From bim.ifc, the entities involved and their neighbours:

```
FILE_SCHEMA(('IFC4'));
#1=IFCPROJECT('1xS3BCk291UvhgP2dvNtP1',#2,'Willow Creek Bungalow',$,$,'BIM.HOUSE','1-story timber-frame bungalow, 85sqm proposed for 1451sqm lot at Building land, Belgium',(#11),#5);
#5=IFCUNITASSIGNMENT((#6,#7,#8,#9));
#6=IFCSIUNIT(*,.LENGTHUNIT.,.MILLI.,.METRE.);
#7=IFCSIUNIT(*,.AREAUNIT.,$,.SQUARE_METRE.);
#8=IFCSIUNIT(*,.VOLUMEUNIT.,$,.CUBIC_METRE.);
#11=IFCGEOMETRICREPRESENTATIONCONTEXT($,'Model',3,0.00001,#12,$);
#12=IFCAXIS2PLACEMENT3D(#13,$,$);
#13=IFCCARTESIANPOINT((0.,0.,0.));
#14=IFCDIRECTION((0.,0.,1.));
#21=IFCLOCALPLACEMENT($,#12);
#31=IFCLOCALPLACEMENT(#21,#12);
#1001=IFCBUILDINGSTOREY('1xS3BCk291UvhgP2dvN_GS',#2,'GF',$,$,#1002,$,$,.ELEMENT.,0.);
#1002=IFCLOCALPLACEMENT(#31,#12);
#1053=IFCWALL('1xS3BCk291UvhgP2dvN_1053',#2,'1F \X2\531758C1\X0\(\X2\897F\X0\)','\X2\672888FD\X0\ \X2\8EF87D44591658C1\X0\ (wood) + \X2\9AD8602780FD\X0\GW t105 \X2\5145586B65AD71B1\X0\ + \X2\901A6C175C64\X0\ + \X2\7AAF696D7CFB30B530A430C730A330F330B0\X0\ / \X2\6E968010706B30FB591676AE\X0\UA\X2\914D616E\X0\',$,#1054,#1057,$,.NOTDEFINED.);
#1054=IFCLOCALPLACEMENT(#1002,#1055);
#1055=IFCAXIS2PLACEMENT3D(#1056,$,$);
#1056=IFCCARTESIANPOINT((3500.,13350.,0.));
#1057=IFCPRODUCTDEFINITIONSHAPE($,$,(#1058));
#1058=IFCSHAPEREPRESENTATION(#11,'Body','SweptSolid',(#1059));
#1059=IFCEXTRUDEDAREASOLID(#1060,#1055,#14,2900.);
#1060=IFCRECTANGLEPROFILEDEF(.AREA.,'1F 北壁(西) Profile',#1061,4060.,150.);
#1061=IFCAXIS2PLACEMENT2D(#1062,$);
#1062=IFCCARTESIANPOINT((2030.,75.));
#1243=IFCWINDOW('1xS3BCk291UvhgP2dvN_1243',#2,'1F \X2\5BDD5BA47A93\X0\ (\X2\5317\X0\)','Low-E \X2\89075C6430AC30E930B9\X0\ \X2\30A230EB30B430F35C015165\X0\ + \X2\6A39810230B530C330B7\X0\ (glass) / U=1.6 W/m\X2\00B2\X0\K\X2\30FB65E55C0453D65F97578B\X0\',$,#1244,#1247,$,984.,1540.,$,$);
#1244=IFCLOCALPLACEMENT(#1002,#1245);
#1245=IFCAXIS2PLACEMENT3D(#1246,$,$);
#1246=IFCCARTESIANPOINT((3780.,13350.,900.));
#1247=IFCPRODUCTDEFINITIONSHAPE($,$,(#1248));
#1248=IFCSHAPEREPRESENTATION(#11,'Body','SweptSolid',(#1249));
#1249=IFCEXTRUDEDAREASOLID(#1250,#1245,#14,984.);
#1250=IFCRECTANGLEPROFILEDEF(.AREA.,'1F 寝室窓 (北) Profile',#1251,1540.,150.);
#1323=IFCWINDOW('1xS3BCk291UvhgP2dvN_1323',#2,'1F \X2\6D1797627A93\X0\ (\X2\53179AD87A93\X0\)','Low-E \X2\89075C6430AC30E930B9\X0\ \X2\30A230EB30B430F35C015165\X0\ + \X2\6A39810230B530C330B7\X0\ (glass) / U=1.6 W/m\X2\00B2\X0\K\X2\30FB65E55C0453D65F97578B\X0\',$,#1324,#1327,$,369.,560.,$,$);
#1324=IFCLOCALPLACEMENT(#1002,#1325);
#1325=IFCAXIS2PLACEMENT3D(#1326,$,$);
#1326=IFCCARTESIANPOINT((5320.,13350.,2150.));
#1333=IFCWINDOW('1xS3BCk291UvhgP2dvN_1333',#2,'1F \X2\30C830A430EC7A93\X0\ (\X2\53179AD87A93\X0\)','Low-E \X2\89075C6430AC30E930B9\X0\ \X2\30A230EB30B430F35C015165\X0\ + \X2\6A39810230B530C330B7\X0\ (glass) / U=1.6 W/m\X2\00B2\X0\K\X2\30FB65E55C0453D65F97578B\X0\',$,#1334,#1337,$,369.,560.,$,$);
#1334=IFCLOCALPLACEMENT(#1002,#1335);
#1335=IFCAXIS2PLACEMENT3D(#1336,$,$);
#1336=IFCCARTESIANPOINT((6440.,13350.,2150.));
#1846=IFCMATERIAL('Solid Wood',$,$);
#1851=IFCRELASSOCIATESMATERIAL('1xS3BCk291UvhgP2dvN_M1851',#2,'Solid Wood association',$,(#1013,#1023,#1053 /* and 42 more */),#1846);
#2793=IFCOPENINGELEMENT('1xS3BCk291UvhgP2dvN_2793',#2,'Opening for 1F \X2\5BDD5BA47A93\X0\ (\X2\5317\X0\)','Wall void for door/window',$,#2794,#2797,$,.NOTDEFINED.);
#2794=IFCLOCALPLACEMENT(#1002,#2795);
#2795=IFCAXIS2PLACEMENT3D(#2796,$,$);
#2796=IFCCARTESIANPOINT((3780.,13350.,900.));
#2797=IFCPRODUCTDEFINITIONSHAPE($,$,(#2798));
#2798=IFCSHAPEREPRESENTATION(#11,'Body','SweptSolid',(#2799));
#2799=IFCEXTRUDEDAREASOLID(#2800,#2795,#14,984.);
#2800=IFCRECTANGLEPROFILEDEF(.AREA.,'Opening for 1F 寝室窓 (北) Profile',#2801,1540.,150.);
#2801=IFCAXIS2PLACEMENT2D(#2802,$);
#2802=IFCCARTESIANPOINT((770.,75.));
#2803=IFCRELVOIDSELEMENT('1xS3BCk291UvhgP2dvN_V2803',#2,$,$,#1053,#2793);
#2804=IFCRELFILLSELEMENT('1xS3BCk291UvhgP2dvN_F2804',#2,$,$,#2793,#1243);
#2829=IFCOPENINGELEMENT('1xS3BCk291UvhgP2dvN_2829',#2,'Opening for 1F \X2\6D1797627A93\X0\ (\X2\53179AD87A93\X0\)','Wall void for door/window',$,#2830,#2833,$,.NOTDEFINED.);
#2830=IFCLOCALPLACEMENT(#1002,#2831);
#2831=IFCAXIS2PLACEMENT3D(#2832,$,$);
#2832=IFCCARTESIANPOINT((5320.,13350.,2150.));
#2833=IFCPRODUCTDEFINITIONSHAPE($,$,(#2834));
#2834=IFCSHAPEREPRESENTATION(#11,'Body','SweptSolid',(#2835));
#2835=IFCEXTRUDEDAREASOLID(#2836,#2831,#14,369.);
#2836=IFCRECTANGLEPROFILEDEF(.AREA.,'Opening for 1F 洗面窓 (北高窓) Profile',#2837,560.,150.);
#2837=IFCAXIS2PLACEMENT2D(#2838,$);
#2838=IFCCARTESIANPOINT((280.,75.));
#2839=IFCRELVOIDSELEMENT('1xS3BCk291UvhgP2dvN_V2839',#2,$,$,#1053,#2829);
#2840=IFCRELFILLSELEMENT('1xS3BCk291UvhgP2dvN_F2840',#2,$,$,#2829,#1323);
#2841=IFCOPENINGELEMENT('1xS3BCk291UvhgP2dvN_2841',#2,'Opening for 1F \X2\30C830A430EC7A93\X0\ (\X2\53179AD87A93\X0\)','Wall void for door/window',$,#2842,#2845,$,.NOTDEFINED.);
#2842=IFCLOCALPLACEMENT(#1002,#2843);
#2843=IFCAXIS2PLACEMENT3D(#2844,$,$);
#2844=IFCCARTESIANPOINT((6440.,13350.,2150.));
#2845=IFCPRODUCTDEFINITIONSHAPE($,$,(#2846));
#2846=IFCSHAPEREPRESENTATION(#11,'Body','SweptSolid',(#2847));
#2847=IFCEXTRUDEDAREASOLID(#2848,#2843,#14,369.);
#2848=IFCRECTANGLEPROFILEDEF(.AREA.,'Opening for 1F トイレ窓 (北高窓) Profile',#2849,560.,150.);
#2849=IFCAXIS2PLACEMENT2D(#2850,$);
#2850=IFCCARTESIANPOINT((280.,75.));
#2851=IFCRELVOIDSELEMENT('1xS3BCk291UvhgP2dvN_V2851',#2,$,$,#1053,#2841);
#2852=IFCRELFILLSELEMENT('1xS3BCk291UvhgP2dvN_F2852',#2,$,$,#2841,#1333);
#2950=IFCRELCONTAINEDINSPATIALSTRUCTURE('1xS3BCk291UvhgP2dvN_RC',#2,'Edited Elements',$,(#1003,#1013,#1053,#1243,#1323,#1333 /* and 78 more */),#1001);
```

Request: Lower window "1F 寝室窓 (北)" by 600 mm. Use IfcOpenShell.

```python
import numpy as np
import ifcopenshell
import ifcopenshell.api.geometry
import ifcopenshell.util.placement
import ifcopenshell.util.unit

model = ifcopenshell.open("bim.ifc")
unit_scale = ifcopenshell.util.unit.calculate_unit_scale(model)

window = model.by_guid("1xS3BCk291UvhgP2dvN_1243")
opening = window.FillsVoids[0].RelatingOpeningElement
dz = -0.6 / unit_scale

shift = np.array([0.0, 0.0, dz])
# The window is not placed relative to its opening, so move both.
for product in (opening, window):
    matrix = ifcopenshell.util.placement.get_local_placement(product.ObjectPlacement)
    matrix[:3, 3] += shift
    ifcopenshell.api.geometry.edit_object_placement(model, product=product, matrix=matrix, is_si=False)

print(f"moved by {dz * unit_scale:+.3f} m")

model.write("bim_rev.ifc")
```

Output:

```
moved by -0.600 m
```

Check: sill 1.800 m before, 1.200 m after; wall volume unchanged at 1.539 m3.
